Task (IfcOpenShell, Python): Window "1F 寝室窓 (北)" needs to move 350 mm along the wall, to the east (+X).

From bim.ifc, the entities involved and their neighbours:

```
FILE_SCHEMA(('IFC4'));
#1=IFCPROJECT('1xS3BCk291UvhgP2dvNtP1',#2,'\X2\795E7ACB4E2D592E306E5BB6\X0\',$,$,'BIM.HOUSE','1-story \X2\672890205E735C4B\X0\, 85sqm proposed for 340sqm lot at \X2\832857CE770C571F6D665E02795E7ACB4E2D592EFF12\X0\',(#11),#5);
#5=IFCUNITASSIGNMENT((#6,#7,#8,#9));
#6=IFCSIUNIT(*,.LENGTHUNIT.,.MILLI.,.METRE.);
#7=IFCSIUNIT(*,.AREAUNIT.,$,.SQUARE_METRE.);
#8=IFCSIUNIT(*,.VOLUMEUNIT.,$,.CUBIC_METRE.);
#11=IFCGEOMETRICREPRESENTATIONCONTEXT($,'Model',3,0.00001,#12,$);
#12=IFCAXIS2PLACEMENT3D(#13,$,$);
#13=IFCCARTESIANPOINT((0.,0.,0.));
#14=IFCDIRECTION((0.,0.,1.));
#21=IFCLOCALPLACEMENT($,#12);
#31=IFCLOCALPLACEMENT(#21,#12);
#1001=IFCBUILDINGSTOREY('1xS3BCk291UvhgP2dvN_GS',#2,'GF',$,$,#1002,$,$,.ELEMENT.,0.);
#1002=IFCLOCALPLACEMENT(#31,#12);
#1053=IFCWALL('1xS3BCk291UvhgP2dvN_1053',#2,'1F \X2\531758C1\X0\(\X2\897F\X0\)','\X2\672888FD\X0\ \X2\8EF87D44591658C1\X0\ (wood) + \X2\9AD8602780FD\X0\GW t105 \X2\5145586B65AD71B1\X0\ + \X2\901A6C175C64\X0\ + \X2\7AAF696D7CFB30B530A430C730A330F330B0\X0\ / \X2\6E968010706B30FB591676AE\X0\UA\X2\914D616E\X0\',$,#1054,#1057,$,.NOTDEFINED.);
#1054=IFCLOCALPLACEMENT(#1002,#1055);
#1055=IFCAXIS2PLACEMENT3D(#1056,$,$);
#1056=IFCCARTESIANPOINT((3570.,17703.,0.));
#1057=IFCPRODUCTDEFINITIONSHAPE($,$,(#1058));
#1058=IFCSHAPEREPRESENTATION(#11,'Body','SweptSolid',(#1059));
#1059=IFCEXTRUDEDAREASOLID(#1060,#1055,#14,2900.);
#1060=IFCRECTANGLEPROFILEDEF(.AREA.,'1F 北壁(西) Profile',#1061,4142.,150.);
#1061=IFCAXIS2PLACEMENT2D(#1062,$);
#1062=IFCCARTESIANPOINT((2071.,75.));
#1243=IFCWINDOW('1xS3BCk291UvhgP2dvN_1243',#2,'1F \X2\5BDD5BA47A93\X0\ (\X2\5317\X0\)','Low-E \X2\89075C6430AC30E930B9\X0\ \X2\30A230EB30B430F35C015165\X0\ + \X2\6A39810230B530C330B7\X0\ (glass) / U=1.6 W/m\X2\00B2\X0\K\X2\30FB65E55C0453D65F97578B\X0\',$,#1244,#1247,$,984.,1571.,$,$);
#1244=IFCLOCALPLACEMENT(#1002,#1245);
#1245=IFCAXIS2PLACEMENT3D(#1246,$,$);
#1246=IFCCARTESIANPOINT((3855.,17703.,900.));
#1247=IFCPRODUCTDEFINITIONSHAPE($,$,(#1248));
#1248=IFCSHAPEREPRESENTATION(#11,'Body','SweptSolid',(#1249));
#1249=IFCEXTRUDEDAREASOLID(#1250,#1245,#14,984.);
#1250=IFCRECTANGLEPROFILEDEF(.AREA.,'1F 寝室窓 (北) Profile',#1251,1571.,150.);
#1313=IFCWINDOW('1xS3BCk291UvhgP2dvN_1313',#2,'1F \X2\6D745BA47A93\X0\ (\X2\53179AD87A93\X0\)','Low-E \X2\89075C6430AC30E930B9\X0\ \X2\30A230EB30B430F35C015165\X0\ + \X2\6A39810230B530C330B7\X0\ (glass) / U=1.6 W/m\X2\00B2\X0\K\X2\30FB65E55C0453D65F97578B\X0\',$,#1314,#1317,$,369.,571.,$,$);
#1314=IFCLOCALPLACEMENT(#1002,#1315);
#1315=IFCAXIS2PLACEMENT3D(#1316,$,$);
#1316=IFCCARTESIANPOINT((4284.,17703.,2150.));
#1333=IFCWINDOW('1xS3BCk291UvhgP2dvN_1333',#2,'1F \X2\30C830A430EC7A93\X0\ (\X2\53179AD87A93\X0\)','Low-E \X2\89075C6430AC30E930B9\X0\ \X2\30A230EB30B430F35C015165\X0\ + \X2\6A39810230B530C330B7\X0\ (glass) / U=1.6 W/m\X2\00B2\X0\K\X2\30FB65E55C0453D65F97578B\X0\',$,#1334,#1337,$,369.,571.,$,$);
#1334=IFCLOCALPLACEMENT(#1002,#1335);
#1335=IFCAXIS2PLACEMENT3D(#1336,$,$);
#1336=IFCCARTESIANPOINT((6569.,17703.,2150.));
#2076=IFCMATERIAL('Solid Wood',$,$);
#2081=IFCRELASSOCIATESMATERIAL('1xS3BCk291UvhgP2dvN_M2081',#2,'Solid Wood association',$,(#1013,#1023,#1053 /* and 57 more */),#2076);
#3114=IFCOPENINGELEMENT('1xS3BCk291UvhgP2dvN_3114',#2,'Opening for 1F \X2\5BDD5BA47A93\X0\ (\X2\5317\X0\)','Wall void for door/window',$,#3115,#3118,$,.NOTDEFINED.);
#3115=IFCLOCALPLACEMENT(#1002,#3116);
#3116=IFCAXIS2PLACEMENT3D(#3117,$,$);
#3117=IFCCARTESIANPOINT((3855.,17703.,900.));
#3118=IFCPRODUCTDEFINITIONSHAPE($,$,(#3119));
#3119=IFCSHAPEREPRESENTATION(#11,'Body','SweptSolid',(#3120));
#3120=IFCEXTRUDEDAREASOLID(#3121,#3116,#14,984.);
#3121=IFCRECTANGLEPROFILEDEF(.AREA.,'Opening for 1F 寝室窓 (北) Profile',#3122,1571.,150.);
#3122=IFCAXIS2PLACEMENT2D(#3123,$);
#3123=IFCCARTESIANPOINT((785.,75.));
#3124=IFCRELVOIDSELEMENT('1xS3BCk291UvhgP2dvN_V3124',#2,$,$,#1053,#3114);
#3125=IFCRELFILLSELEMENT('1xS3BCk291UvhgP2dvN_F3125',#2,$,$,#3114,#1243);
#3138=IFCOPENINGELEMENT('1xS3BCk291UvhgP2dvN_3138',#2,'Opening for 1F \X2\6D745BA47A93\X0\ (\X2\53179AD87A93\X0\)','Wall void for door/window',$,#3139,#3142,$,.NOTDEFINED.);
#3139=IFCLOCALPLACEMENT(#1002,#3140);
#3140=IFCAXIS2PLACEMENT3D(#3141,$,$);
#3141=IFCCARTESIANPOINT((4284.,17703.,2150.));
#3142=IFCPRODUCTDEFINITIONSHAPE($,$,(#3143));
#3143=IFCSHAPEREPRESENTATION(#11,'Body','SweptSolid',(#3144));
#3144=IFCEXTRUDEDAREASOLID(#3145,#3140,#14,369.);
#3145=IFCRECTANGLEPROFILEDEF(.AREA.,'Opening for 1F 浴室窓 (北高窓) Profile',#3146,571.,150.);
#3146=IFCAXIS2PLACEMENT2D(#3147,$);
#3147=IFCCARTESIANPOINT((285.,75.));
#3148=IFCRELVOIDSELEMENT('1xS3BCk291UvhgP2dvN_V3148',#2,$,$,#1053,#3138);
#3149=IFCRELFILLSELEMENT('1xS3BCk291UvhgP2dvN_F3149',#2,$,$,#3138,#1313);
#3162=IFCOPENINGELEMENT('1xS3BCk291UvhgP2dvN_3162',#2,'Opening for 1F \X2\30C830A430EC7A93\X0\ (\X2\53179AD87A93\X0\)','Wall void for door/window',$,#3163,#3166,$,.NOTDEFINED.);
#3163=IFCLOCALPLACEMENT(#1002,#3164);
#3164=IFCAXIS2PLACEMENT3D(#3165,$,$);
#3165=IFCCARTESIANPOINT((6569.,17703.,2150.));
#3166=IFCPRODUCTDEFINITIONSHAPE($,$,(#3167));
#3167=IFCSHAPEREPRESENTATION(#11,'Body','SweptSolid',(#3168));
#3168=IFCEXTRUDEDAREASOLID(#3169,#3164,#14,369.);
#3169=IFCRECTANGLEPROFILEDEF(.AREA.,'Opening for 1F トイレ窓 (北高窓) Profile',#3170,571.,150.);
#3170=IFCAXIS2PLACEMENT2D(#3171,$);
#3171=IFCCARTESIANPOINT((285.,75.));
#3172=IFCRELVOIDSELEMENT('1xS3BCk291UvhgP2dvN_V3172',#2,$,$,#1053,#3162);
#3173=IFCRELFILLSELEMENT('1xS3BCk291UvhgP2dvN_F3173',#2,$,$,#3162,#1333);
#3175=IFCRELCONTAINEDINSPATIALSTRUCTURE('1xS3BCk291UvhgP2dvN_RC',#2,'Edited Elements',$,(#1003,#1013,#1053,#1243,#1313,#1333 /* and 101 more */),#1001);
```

```python
import ifcopenshell
import ifcopenshell.api.geometry
import ifcopenshell.util.placement
import ifcopenshell.util.unit

model = ifcopenshell.open("bim.ifc")
unit_scale = ifcopenshell.util.unit.calculate_unit_scale(model)

window = model.by_guid("1xS3BCk291UvhgP2dvN_1243")
opening = window.FillsVoids[0].RelatingOpeningElement
wall = opening.VoidsElements[0].RelatingBuildingElement

wall_matrix = ifcopenshell.util.placement.get_local_placement(wall.ObjectPlacement)
shift = wall_matrix[:3, 0] * 0.35 / unit_scale
before = ifcopenshell.util.placement.get_local_placement(window.ObjectPlacement)[:3, 3].copy()

# The window is not placed relative to its opening, so move both.
for product in (opening, window):
    matrix = ifcopenshell.util.placement.get_local_placement(product.ObjectPlacement)
    matrix[:3, 3] += shift
    ifcopenshell.api.geometry.edit_object_placement(model, product=product, matrix=matrix, is_si=False)

after = ifcopenshell.util.placement.get_local_placement(window.ObjectPlacement)[:3, 3]
print("window moved by", (after - before).round(3) + 0.0)

model.write("bim_updated.ifc")
```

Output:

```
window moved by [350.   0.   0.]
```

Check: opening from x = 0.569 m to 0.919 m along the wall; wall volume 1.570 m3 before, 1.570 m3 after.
